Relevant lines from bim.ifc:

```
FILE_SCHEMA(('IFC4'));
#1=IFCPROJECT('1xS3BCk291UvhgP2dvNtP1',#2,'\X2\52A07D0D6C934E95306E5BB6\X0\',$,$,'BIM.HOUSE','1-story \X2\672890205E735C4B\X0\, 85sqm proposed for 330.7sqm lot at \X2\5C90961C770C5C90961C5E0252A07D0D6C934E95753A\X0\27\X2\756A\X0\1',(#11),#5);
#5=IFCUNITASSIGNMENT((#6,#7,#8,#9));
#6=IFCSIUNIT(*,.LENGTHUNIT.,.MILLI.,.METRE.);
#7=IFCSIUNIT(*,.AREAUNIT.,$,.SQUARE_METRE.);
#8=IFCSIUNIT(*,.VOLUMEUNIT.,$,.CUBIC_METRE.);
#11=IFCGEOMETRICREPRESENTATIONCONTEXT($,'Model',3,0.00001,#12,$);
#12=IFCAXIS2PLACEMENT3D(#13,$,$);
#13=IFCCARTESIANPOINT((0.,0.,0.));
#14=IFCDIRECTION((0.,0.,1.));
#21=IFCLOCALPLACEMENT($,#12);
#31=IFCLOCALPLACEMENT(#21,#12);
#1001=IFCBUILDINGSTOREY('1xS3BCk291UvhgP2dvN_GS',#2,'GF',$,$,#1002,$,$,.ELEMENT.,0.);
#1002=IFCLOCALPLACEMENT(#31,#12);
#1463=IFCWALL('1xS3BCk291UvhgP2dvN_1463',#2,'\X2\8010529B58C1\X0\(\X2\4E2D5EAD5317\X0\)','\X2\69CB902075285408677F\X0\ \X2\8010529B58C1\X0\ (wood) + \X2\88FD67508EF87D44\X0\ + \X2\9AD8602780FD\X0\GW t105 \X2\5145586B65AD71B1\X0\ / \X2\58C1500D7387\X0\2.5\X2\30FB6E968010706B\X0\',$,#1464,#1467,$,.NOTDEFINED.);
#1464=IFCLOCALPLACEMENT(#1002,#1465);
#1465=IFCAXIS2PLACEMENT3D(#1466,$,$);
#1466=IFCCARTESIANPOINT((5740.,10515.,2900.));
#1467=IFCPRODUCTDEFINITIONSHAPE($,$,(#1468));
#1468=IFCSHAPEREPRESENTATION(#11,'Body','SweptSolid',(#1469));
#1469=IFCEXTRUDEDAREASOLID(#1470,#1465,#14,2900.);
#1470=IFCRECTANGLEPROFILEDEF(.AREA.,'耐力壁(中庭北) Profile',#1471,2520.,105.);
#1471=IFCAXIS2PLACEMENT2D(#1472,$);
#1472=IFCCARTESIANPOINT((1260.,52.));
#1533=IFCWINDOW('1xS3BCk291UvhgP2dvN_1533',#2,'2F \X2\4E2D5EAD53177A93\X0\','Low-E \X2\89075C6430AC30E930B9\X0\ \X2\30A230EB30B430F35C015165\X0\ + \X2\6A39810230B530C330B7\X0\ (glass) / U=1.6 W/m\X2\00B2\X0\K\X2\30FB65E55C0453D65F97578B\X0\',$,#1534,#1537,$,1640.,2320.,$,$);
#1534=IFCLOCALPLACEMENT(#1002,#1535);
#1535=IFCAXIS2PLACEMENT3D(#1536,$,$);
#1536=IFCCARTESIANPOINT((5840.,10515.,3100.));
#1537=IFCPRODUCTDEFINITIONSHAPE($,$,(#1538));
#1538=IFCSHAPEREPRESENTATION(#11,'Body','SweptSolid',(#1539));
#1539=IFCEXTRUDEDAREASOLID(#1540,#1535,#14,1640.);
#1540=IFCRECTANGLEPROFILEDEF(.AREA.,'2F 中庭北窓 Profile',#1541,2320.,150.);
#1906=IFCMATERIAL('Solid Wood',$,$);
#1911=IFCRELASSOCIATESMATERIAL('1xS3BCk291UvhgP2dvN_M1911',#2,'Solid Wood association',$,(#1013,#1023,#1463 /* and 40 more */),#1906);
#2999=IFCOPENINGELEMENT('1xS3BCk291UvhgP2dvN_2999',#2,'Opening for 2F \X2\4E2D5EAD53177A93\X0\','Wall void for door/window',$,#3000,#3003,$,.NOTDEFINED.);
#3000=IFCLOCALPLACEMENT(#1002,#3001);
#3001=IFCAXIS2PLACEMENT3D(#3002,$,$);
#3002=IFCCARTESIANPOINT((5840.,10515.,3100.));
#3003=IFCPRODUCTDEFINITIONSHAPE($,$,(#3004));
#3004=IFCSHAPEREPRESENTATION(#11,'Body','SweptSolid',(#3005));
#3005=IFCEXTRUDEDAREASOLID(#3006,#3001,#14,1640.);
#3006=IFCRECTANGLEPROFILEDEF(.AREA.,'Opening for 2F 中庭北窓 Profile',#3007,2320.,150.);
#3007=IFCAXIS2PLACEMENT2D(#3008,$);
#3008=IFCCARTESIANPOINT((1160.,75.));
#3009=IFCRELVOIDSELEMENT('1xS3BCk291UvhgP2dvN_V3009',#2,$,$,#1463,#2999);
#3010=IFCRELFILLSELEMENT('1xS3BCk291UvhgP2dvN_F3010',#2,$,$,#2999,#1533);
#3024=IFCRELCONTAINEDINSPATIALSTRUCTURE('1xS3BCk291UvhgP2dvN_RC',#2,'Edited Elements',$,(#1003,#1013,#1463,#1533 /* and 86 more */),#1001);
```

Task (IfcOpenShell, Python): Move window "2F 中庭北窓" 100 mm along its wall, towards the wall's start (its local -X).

```python
import ifcopenshell
import ifcopenshell.api.geometry
import ifcopenshell.util.placement

model = ifcopenshell.open("bim.ifc")

window = model.by_guid("1xS3BCk291UvhgP2dvN_1533")
opening = window.FillsVoids[0].RelatingOpeningElement
wall = opening.VoidsElements[0].RelatingBuildingElement

wall_matrix = ifcopenshell.util.placement.get_local_placement(wall.ObjectPlacement)
shift = wall_matrix[:3, 0] * -100.0
before = ifcopenshell.util.placement.get_local_placement(window.ObjectPlacement)[:3, 3].copy()

# The window is not placed relative to its opening, so move both.
for product in (opening, window):
    matrix = ifcopenshell.util.placement.get_local_placement(product.ObjectPlacement)
    matrix[:3, 3] += shift
    ifcopenshell.api.geometry.edit_object_placement(model, product=product, matrix=matrix, is_si=False)

after = ifcopenshell.util.placement.get_local_placement(window.ObjectPlacement)[:3, 3]
print("window moved by", (after - before).round(3) + 0.0)

model.write("bim-out.ifc")
```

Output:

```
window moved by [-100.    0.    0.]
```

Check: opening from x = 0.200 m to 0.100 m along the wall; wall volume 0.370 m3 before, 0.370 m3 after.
